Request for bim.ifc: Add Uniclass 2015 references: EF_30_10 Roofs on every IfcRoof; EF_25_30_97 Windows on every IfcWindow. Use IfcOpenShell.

First a look at what the model holds.

```python
import ifcopenshell

model = ifcopenshell.open("bim.ifc")
print(model.schema)
print("classifications:", [c.Name for c in model.by_type("IfcClassification")])
for ifc_class in ("IfcDoor", "IfcRoof", "IfcStair", "IfcWall", "IfcWindow"):
    print(ifc_class, len(model.by_type(ifc_class)))
```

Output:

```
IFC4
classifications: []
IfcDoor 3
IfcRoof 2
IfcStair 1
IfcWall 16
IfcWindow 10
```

```python
import ifcopenshell
import ifcopenshell.api.classification

model = ifcopenshell.open("bim.ifc")

system = ifcopenshell.api.classification.add_classification(model, classification="Uniclass 2015")

codes = {
    "IfcRoof": ("EF_30_10", "Roofs"),
    "IfcWindow": ("EF_25_30_97", "Windows"),
}
for ifc_class, (code, name) in codes.items():
    products = model.by_type(ifc_class)
    ifcopenshell.api.classification.add_reference(
        model, products=products, classification=system, identification=code, name=name
    )
    print(code, len(products))

model.write("bim_v2.ifc")
```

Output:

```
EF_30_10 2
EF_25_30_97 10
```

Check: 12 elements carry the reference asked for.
